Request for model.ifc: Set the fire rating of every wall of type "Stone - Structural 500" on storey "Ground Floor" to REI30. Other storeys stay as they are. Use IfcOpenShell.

First a look at what the model holds.

```python
import ifcopenshell
import ifcopenshell.util.element

model = ifcopenshell.open("model.ifc")
print(model.schema)
storey = next(s for s in model.by_type("IfcBuildingStorey") if s.Name == "Ground Floor")
walls = [e for e in ifcopenshell.util.element.get_decomposition(storey) if e.is_a("IfcWall")]
seen = {}
for e in walls:
    element_type = ifcopenshell.util.element.get_type(e)
    key = (element_type.Name if element_type != e and element_type else None, ifcopenshell.util.element.get_pset(e, "Pset_WallCommon", "FireRating"))
    seen[key] = seen.get(key, 0) + 1
for (name, value), count in sorted(seen.items(), key=str):
    print(count, "x", name, "|", value)
```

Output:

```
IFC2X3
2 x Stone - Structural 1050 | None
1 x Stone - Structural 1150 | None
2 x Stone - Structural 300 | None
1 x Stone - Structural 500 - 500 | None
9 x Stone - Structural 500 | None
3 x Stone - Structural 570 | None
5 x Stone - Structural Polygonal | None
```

```python
import ifcopenshell
import ifcopenshell.api.pset
import ifcopenshell.util.element

model = ifcopenshell.open("model.ifc")

storey = next(s for s in model.by_type("IfcBuildingStorey") if s.Name == "Ground Floor")
walls = [e for e in ifcopenshell.util.element.get_decomposition(storey) if e.is_a("IfcWall")]

count = 0
for e in walls:
    element_type = ifcopenshell.util.element.get_type(e)
    if element_type in (None, e) or element_type.Name != "Stone - Structural 500":
        continue
    # add_pset returns the element's existing set when there is one.
    pset = ifcopenshell.api.pset.add_pset(model, product=e, name="Pset_WallCommon")
    ifcopenshell.api.pset.edit_pset(model, pset=pset, properties={"FireRating": "REI30"})
    count += 1

print(count, "walls updated")

model.write("model_edited.ifc")
```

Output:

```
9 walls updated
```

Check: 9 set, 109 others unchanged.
